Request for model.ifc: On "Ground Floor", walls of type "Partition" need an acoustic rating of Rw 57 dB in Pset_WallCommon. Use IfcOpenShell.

First a look at what the model holds.

```python
import ifcopenshell
import ifcopenshell.util.element

model = ifcopenshell.open("model.ifc")
print(model.schema)
storey = next(s for s in model.by_type("IfcBuildingStorey") if s.Name == "Ground Floor")
walls = [e for e in ifcopenshell.util.element.get_decomposition(storey) if e.is_a("IfcWall")]
seen = {}
for e in walls:
    element_type = ifcopenshell.util.element.get_type(e)
    key = (element_type.Name if element_type != e and element_type else None, ifcopenshell.util.element.get_pset(e, "Pset_WallCommon", "AcousticRating"))
    seen[key] = seen.get(key, 0) + 1
for (name, value), count in sorted(seen.items(), key=str):
    print(count, "x", name, "|", value)
```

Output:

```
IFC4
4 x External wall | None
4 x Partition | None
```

```python
import ifcopenshell
import ifcopenshell.api.pset
import ifcopenshell.util.element

model = ifcopenshell.open("model.ifc")

storey = next(s for s in model.by_type("IfcBuildingStorey") if s.Name == "Ground Floor")
walls = [e for e in ifcopenshell.util.element.get_decomposition(storey) if e.is_a("IfcWall")]

count = 0
for e in walls:
    element_type = ifcopenshell.util.element.get_type(e)
    if element_type in (None, e) or element_type.Name != "Partition":
        continue
    # add_pset returns the element's existing set when there is one.
    pset = ifcopenshell.api.pset.add_pset(model, product=e, name="Pset_WallCommon")
    ifcopenshell.api.pset.edit_pset(model, pset=pset, properties={"AcousticRating": "Rw 57 dB"})
    count += 1

print(count, "walls updated")

model.write("model_updated.ifc")
```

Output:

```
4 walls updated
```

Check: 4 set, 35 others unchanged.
